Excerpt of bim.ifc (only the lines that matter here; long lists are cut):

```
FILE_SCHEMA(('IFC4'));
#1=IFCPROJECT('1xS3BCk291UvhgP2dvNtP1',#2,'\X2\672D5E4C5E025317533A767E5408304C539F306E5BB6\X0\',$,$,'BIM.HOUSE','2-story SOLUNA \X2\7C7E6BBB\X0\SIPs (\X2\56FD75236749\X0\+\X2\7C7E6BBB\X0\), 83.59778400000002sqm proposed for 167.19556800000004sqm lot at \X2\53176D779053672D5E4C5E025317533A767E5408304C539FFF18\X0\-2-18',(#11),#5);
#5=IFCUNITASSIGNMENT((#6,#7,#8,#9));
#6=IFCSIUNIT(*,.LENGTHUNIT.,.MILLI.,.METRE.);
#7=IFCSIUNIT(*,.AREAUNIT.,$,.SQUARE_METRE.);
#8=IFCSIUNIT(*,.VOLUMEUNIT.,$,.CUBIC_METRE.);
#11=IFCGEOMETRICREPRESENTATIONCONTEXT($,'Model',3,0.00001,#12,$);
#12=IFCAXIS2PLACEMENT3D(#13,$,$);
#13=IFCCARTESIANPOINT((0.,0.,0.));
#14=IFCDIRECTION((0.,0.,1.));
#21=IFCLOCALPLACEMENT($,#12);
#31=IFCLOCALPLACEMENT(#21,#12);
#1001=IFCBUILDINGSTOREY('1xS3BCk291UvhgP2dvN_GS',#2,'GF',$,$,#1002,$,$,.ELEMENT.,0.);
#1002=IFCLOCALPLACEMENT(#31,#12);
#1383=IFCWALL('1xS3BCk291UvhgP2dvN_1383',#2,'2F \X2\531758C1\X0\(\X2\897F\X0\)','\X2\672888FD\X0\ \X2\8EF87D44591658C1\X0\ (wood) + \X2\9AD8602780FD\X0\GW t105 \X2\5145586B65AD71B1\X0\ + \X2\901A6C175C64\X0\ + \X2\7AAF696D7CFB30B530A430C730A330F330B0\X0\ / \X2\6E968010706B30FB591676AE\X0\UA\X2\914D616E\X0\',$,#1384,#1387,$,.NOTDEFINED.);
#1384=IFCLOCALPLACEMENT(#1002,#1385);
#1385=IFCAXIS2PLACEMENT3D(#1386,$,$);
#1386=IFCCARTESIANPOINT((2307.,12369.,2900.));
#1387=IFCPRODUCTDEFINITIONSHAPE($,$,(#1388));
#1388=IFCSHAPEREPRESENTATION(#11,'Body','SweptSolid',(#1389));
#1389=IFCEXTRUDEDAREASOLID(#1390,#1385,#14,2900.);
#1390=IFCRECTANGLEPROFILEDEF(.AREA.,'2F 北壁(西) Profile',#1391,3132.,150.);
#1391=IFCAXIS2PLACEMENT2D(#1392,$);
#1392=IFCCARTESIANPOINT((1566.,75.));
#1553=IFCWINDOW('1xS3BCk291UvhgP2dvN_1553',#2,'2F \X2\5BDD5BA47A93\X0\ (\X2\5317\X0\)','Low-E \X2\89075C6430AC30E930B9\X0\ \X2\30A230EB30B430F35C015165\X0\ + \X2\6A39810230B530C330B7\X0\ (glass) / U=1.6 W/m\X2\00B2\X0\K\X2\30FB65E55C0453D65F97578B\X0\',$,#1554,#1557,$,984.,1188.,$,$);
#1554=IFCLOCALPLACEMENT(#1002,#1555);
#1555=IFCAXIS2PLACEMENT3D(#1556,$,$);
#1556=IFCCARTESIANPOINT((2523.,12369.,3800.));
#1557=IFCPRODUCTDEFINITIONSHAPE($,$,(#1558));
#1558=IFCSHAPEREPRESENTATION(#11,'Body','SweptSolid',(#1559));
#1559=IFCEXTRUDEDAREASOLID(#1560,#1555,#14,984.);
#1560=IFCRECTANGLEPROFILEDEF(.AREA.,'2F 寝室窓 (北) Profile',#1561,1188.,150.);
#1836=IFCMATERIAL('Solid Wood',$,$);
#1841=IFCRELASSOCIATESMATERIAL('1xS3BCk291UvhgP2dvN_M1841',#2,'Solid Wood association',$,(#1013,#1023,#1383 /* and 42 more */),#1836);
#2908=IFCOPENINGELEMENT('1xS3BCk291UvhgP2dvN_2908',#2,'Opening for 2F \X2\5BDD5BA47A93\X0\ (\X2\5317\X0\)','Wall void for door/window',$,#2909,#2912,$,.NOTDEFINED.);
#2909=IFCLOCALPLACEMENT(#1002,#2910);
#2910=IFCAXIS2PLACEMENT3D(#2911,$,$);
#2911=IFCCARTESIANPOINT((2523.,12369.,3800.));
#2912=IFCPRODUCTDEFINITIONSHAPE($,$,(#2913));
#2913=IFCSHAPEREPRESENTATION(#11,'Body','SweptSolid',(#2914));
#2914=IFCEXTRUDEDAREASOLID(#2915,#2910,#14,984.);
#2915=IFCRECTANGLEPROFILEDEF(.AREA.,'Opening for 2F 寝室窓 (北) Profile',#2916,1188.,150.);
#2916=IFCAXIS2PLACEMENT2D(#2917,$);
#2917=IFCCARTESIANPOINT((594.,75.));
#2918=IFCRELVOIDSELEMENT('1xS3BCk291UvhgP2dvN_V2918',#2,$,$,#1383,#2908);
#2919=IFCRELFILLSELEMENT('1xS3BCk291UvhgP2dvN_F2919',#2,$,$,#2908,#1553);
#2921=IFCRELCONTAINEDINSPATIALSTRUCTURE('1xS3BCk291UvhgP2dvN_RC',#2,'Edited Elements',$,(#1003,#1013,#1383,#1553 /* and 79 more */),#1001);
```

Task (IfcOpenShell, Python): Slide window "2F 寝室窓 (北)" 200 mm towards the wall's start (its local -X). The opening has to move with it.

```python
import ifcopenshell
import ifcopenshell.api.geometry
import ifcopenshell.util.placement
import ifcopenshell.util.unit

model = ifcopenshell.open("bim.ifc")
unit_scale = ifcopenshell.util.unit.calculate_unit_scale(model)

window = model.by_guid("1xS3BCk291UvhgP2dvN_1553")
opening = window.FillsVoids[0].RelatingOpeningElement
wall = opening.VoidsElements[0].RelatingBuildingElement

wall_matrix = ifcopenshell.util.placement.get_local_placement(wall.ObjectPlacement)
shift = wall_matrix[:3, 0] * -0.2 / unit_scale
before = ifcopenshell.util.placement.get_local_placement(window.ObjectPlacement)[:3, 3].copy()

# The window is not placed relative to its opening, so move both.
for product in (opening, window):
    matrix = ifcopenshell.util.placement.get_local_placement(product.ObjectPlacement)
    matrix[:3, 3] += shift
    ifcopenshell.api.geometry.edit_object_placement(model, product=product, matrix=matrix, is_si=False)

after = ifcopenshell.util.placement.get_local_placement(window.ObjectPlacement)[:3, 3]
print("window moved by", (after - before).round(3) + 0.0)

model.write("bim_updated.ifc")
```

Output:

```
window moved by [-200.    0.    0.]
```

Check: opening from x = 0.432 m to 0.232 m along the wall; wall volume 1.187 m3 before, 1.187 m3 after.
